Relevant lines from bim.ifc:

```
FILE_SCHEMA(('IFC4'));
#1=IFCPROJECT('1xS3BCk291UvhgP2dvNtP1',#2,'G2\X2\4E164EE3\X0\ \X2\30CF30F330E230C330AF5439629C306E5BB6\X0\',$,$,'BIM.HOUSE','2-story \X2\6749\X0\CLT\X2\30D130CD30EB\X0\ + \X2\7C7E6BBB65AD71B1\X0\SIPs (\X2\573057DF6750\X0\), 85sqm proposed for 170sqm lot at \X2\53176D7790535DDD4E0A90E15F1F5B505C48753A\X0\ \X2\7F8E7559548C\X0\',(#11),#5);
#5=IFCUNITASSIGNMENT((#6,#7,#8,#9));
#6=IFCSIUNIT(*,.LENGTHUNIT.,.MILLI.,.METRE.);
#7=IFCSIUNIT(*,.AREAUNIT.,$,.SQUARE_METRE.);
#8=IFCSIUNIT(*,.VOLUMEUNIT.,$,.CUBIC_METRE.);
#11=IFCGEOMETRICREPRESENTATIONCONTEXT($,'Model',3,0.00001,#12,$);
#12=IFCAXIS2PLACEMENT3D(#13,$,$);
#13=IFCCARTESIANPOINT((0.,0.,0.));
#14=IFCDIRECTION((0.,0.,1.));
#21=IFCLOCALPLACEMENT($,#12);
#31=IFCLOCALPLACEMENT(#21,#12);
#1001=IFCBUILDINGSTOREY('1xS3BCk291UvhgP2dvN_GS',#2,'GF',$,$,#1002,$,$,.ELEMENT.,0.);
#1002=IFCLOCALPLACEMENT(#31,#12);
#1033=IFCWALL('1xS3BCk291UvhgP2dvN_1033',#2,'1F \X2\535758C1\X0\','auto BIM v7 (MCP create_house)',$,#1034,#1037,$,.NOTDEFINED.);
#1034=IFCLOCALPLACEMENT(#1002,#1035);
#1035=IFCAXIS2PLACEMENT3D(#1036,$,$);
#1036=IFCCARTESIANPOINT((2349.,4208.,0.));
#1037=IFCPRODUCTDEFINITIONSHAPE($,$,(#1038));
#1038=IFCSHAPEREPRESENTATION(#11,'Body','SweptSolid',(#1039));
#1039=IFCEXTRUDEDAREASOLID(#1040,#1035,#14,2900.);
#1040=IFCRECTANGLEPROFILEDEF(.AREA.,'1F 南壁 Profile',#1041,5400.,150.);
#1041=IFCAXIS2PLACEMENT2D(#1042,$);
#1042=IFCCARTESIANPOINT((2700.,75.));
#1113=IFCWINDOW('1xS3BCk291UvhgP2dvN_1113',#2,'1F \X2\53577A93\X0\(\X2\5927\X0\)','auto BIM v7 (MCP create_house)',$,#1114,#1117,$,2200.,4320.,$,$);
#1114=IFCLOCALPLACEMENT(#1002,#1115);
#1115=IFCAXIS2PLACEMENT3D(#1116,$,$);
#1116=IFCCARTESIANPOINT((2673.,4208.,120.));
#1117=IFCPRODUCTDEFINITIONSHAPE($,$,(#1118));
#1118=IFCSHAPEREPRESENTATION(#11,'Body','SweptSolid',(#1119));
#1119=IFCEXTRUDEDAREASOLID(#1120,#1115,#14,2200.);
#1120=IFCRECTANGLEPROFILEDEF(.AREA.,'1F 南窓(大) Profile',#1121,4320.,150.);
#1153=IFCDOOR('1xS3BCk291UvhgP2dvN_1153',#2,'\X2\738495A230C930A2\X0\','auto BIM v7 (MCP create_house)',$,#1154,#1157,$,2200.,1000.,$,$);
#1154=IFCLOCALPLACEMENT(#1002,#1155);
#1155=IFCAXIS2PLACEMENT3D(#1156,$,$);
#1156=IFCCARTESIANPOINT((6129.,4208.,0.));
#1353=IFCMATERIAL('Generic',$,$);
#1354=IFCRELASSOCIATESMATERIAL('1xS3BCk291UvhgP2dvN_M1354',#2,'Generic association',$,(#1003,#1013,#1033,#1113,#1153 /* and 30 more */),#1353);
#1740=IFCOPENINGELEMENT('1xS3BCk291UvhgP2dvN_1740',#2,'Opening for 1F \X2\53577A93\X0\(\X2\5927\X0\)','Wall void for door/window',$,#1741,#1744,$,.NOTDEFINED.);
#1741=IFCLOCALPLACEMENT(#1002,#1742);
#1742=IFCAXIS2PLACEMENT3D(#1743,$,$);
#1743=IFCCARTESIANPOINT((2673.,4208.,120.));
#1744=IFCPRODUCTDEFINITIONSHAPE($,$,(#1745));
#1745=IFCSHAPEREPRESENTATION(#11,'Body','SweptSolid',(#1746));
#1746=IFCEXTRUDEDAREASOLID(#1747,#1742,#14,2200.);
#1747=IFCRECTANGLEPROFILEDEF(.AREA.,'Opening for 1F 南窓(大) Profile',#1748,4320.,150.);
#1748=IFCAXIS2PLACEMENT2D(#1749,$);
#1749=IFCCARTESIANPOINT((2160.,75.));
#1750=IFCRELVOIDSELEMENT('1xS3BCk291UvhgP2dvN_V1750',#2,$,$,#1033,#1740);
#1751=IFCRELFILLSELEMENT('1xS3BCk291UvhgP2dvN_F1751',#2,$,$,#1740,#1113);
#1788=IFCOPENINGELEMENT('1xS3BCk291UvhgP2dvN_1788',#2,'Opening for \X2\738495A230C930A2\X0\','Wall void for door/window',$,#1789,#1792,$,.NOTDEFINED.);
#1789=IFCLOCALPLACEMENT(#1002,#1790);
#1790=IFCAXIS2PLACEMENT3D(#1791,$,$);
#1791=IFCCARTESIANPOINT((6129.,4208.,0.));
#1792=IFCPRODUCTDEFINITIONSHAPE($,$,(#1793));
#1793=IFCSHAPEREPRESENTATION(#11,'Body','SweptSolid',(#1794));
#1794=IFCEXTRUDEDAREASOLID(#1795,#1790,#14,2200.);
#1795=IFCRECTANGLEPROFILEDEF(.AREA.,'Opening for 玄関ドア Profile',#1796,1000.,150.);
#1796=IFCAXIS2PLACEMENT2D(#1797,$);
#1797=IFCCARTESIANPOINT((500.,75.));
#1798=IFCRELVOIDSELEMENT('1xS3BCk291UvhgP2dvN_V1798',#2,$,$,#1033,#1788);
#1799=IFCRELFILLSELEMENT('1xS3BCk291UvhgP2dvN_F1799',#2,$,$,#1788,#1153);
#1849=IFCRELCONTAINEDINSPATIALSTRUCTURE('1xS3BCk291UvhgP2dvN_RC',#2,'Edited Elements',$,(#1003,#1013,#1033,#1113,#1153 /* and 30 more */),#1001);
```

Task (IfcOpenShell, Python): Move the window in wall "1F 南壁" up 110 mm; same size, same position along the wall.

```python
import numpy as np
import ifcopenshell
import ifcopenshell.api.geometry
import ifcopenshell.util.placement
import ifcopenshell.util.unit

model = ifcopenshell.open("bim.ifc")
unit_scale = ifcopenshell.util.unit.calculate_unit_scale(model)

window = model.by_guid("1xS3BCk291UvhgP2dvN_1113")
opening = window.FillsVoids[0].RelatingOpeningElement
dz = 0.11 / unit_scale

shift = np.array([0.0, 0.0, dz])
# The window is not placed relative to its opening, so move both.
for product in (opening, window):
    matrix = ifcopenshell.util.placement.get_local_placement(product.ObjectPlacement)
    matrix[:3, 3] += shift
    ifcopenshell.api.geometry.edit_object_placement(model, product=product, matrix=matrix, is_si=False)

print(f"moved by {dz * unit_scale:+.3f} m")

model.write("bim_rev.ifc")
```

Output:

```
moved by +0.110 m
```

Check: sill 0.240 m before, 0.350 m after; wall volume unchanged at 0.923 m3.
